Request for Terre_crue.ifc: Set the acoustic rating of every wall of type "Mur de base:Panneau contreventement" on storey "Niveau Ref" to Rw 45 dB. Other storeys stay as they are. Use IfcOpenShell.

First a look at what the model holds.

```python
import ifcopenshell
import ifcopenshell.util.element

model = ifcopenshell.open("Terre_crue.ifc")
print(model.schema)
storey = next(s for s in model.by_type("IfcBuildingStorey") if s.Name == "Niveau Ref")
walls = [e for e in ifcopenshell.util.element.get_decomposition(storey) if e.is_a("IfcWall")]
seen = {}
for e in walls:
    element_type = ifcopenshell.util.element.get_type(e)
    key = (element_type.Name if element_type != e and element_type else None, ifcopenshell.util.element.get_pset(e, "Pset_WallCommon", "AcousticRating"))
    seen[key] = seen.get(key, 0) + 1
for (name, value), count in sorted(seen.items(), key=str):
    print(count, "x", name, "|", value)
```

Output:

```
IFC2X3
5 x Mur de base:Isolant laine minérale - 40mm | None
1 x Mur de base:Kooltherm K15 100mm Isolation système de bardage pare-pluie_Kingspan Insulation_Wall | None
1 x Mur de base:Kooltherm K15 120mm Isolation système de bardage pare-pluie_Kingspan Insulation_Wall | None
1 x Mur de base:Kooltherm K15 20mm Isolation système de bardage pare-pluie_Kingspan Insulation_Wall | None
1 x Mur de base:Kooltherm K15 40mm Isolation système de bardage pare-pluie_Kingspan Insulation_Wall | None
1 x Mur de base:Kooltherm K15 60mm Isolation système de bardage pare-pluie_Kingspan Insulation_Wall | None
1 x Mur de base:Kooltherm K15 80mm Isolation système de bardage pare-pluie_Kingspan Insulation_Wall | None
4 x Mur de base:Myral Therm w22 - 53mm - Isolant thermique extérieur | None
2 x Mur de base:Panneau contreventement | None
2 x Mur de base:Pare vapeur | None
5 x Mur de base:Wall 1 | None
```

```python
import ifcopenshell
import ifcopenshell.api.pset
import ifcopenshell.util.element

model = ifcopenshell.open("Terre_crue.ifc")

storey = next(s for s in model.by_type("IfcBuildingStorey") if s.Name == "Niveau Ref")
walls = [e for e in ifcopenshell.util.element.get_decomposition(storey) if e.is_a("IfcWall")]

count = 0
for e in walls:
    element_type = ifcopenshell.util.element.get_type(e)
    if element_type in (None, e) or element_type.Name != "Mur de base:Panneau contreventement":
        continue
    # add_pset returns the element's existing set when there is one.
    pset = ifcopenshell.api.pset.add_pset(model, product=e, name="Pset_WallCommon")
    ifcopenshell.api.pset.edit_pset(model, pset=pset, properties={"AcousticRating": "Rw 45 dB"})
    count += 1

print(count, "walls updated")

model.write("Terre_crue_rev.ifc")
```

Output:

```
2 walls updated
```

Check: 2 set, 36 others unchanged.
